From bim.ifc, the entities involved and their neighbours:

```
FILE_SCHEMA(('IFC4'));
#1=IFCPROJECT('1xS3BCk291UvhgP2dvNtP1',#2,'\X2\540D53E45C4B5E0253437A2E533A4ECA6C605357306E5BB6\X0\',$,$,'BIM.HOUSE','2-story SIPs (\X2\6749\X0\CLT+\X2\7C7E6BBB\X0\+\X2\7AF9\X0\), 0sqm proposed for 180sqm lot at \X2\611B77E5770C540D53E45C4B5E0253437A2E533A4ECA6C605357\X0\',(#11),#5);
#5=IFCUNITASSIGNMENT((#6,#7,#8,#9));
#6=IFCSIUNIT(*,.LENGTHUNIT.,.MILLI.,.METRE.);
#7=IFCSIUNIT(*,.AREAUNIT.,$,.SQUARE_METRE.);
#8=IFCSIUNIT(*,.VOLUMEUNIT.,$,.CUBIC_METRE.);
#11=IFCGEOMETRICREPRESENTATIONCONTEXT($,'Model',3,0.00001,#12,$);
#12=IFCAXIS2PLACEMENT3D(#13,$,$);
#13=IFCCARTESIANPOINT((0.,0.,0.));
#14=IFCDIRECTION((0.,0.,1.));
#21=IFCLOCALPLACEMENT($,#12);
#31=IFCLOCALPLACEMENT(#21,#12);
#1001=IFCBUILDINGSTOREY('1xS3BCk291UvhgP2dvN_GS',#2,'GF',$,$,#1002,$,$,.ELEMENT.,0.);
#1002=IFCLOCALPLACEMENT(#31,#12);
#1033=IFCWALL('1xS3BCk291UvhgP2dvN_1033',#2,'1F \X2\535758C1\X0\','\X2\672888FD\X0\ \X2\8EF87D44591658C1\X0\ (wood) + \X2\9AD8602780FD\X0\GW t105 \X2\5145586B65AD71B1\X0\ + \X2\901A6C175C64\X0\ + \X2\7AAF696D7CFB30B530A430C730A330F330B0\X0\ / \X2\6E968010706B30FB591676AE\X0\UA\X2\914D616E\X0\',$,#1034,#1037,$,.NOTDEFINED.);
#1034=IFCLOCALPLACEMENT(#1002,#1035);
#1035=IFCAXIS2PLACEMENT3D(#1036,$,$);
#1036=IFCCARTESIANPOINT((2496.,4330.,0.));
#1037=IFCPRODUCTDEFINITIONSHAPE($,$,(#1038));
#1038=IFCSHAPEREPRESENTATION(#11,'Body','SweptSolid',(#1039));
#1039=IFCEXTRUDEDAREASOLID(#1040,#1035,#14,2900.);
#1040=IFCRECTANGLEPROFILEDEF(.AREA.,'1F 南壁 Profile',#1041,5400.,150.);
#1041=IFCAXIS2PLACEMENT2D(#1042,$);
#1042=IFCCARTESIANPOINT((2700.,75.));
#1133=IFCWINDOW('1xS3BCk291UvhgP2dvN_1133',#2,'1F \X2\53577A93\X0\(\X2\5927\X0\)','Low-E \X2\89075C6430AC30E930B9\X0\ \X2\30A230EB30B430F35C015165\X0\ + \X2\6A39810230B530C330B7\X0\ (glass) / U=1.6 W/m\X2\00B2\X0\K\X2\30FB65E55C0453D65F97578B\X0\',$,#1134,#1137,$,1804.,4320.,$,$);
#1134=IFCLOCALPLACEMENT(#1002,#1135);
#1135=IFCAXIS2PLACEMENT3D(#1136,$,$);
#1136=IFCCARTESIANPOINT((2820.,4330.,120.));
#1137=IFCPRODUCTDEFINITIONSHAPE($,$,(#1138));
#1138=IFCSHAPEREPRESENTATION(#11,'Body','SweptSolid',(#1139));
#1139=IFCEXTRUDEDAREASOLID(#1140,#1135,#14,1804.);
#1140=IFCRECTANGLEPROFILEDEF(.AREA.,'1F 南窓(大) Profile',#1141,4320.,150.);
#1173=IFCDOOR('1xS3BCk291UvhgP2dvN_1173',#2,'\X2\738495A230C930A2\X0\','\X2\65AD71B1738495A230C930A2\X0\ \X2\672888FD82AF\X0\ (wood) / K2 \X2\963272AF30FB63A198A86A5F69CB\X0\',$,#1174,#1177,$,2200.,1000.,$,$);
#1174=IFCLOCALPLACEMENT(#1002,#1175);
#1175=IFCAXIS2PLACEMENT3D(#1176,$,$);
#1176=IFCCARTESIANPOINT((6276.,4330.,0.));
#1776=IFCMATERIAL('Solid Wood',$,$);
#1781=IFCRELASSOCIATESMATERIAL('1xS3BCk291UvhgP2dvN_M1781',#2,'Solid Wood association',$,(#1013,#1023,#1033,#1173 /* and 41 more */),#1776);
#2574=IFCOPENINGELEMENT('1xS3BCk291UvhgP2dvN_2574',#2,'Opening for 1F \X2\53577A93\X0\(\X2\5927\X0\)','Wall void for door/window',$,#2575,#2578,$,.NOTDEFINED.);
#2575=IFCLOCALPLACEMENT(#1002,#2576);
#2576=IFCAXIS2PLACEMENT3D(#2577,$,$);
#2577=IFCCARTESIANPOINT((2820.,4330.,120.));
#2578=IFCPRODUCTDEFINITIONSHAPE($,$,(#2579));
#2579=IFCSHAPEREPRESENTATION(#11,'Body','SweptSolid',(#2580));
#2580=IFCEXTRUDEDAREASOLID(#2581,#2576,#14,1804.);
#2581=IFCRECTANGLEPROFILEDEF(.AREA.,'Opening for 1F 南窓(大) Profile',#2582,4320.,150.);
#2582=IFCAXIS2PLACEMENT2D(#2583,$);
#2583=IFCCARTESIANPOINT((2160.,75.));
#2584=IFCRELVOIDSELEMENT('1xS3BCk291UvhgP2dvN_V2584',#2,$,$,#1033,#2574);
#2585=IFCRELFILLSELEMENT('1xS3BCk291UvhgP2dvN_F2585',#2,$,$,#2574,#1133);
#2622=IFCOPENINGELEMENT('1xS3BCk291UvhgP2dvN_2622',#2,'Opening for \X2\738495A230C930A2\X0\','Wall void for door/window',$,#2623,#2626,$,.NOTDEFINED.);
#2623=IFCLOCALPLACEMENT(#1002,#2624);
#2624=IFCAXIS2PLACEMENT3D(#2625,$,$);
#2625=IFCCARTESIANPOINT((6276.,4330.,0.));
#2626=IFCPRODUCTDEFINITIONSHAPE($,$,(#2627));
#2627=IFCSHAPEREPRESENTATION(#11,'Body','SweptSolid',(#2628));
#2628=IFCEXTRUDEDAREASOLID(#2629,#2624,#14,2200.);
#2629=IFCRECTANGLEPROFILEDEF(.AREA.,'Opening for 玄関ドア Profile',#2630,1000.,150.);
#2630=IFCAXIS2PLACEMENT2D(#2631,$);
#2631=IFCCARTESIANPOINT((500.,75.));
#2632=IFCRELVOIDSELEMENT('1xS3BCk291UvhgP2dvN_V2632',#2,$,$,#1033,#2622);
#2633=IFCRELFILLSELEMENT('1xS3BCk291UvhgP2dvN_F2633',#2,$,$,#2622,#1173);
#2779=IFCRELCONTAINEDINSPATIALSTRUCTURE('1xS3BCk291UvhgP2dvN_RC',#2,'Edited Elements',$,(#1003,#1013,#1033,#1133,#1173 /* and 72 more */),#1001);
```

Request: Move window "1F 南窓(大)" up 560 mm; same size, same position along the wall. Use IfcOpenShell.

```python
import numpy as np
import ifcopenshell
import ifcopenshell.api.geometry
import ifcopenshell.util.placement
import ifcopenshell.util.unit

model = ifcopenshell.open("bim.ifc")
unit_scale = ifcopenshell.util.unit.calculate_unit_scale(model)

window = model.by_guid("1xS3BCk291UvhgP2dvN_1133")
opening = window.FillsVoids[0].RelatingOpeningElement
dz = 560.0

shift = np.array([0.0, 0.0, dz])
# The window is not placed relative to its opening, so move both.
for product in (opening, window):
    matrix = ifcopenshell.util.placement.get_local_placement(product.ObjectPlacement)
    matrix[:3, 3] += shift
    ifcopenshell.api.geometry.edit_object_placement(model, product=product, matrix=matrix, is_si=False)

print(f"moved by {dz * unit_scale:+.3f} m")

model.write("bim_updated.ifc")
```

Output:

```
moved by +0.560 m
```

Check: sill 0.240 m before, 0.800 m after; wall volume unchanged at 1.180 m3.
